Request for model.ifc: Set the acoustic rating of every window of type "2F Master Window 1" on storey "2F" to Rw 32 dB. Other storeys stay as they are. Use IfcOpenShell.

First a look at what the model holds.

```python
import ifcopenshell
import ifcopenshell.util.element

model = ifcopenshell.open("model.ifc")
print(model.schema)
storey = next(s for s in model.by_type("IfcBuildingStorey") if s.Name == "2F")
windows = [e for e in ifcopenshell.util.element.get_decomposition(storey) if e.is_a("IfcWindow")]
seen = {}
for e in windows:
    element_type = ifcopenshell.util.element.get_type(e)
    key = (element_type.Name if element_type != e and element_type else None, ifcopenshell.util.element.get_pset(e, "Pset_WindowCommon", "AcousticRating"))
    seen[key] = seen.get(key, 0) + 1
for (name, value), count in sorted(seen.items(), key=str):
    print(count, "x", name, "|", value)
```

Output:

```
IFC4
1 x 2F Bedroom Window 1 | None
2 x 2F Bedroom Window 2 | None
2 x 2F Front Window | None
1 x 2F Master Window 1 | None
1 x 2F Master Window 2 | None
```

```python
import ifcopenshell
import ifcopenshell.api.pset
import ifcopenshell.util.element

model = ifcopenshell.open("model.ifc")

storey = next(s for s in model.by_type("IfcBuildingStorey") if s.Name == "2F")
windows = [e for e in ifcopenshell.util.element.get_decomposition(storey) if e.is_a("IfcWindow")]

count = 0
for e in windows:
    element_type = ifcopenshell.util.element.get_type(e)
    if element_type in (None, e) or element_type.Name != "2F Master Window 1":
        continue
    # add_pset returns the element's existing set when there is one.
    pset = ifcopenshell.api.pset.add_pset(model, product=e, name="Pset_WindowCommon")
    ifcopenshell.api.pset.edit_pset(model, pset=pset, properties={"AcousticRating": "Rw 32 dB"})
    count += 1

print(count, "windows updated")

model.write("model_rev.ifc")
```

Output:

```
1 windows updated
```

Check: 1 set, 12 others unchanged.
